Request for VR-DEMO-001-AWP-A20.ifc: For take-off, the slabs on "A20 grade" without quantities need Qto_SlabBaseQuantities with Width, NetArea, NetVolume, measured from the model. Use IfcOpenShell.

First a look at what the model holds.

```python
import ifcopenshell
import ifcopenshell.util.element
import ifcopenshell.util.unit

model = ifcopenshell.open("VR-DEMO-001-AWP-A20.ifc")
print(model.schema)
for unit_type in ("LENGTHUNIT", "AREAUNIT", "VOLUMEUNIT"):
    print(unit_type, ifcopenshell.util.unit.calculate_unit_scale(model, unit_type))
storey = next(s for s in model.by_type("IfcBuildingStorey") if s.Name == "A20 grade")
slabs = [e for e in ifcopenshell.util.element.get_decomposition(storey) if e.is_a("IfcSlab")]
for e in sorted(slabs, key=lambda e: e.id()):
    print(e.id(), e.is_a(), e.Name, list(ifcopenshell.util.element.get_psets(e, qtos_only=True)), sep=" | ")
```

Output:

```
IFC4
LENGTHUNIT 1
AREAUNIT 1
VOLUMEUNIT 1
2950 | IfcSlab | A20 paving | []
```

```python
import ifcopenshell
import ifcopenshell.api.pset
import ifcopenshell.geom
import ifcopenshell.util.element
import ifcopenshell.util.shape
import ifcopenshell.util.unit

model = ifcopenshell.open("VR-DEMO-001-AWP-A20.ifc")
unit_scale = ifcopenshell.util.unit.calculate_unit_scale(model)
area_scale = ifcopenshell.util.unit.calculate_unit_scale(model, "AREAUNIT")
volume_scale = ifcopenshell.util.unit.calculate_unit_scale(model, "VOLUMEUNIT")
settings = ifcopenshell.geom.settings()

storey = next(s for s in model.by_type("IfcBuildingStorey") if s.Name == "A20 grade")
slabs = [e for e in ifcopenshell.util.element.get_decomposition(storey) if e.is_a("IfcSlab")]

for e in sorted(slabs, key=lambda e: e.id()):
    if ifcopenshell.util.element.get_psets(e, qtos_only=True, should_inherit=False):
        continue
    # Geometry comes back in metres, in the element's own axes.
    shape = ifcopenshell.geom.create_shape(settings, e)
    values = {
        "Width": ifcopenshell.util.shape.get_z(shape.geometry) / unit_scale,
        "NetArea": ifcopenshell.util.shape.get_footprint_area(shape.geometry) / area_scale,
        "NetVolume": ifcopenshell.util.shape.get_volume(shape.geometry) / volume_scale,
    }
    qto = ifcopenshell.api.pset.add_qto(model, product=e, name="Qto_SlabBaseQuantities")
    ifcopenshell.api.pset.edit_qto(model, qto=qto, properties=values)
    print(e.id(), {k: round(v, 3) for k, v in values.items()})

model.write("VR-DEMO-001-AWP-A20_rev.ifc")
```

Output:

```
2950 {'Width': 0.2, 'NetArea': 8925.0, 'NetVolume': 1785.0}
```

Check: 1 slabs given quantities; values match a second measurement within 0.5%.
